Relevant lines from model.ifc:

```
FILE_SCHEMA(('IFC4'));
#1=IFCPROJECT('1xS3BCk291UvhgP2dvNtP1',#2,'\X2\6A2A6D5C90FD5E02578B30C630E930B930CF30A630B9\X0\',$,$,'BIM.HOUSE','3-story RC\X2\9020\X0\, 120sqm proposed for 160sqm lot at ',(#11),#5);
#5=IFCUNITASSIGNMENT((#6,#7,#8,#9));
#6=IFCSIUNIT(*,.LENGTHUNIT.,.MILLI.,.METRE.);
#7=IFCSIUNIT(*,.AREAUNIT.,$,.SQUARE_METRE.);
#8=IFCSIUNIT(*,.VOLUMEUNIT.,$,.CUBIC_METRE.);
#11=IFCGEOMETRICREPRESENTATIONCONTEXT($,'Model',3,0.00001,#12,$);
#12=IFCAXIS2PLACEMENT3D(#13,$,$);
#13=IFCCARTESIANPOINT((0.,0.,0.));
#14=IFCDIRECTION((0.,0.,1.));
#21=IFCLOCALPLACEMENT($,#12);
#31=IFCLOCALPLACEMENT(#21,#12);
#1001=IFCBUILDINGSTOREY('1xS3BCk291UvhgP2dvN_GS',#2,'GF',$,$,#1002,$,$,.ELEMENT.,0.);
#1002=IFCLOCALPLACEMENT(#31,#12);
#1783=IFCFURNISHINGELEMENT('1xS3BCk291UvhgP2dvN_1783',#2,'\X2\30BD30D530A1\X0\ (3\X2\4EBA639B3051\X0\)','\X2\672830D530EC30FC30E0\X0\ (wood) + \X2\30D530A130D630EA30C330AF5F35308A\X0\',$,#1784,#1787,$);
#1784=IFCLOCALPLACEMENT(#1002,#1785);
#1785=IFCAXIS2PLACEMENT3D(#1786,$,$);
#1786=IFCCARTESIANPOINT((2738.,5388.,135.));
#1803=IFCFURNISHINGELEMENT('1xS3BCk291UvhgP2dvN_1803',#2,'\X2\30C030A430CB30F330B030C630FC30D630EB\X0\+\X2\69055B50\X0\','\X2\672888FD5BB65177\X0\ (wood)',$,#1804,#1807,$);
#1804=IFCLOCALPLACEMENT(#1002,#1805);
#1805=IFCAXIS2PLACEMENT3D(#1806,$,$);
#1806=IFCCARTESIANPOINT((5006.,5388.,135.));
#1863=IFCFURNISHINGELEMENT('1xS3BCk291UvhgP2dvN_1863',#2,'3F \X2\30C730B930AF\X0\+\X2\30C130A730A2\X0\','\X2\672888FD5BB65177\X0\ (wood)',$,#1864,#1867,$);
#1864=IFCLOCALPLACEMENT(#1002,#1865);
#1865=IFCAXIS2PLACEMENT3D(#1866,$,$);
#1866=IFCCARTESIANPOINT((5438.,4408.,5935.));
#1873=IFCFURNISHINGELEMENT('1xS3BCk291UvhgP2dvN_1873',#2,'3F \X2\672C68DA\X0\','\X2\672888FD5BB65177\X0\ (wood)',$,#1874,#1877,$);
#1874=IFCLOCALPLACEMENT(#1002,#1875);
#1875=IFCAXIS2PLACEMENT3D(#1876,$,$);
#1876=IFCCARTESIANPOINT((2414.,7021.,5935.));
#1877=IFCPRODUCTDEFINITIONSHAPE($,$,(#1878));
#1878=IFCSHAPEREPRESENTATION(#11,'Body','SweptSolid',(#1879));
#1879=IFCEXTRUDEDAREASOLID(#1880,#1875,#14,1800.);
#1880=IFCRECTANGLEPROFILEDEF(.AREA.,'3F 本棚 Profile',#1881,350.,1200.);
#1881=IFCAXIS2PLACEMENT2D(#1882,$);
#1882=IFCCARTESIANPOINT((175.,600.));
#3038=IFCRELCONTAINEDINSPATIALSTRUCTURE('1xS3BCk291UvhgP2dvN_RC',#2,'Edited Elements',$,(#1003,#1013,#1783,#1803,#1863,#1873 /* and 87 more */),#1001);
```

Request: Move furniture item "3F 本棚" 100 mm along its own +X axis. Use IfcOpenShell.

```python
import ifcopenshell
import ifcopenshell.api.geometry
import ifcopenshell.util.placement
import ifcopenshell.util.unit

model = ifcopenshell.open("model.ifc")
unit_scale = ifcopenshell.util.unit.calculate_unit_scale(model)

item = model.by_guid("1xS3BCk291UvhgP2dvN_1873")
matrix = ifcopenshell.util.placement.get_local_placement(item.ObjectPlacement)
matrix[:3, 3] += matrix[:3, 0] * 0.1 / unit_scale
ifcopenshell.api.geometry.edit_object_placement(model, product=item, matrix=matrix, is_si=False)

print(ifcopenshell.util.placement.get_local_placement(item.ObjectPlacement).round(3) + 0.0)

model.write("model_rev.ifc")
```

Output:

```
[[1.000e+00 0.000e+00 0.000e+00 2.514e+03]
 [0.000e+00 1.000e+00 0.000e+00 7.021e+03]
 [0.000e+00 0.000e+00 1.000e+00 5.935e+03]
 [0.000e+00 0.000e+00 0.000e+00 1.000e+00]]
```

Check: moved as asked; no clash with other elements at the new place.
